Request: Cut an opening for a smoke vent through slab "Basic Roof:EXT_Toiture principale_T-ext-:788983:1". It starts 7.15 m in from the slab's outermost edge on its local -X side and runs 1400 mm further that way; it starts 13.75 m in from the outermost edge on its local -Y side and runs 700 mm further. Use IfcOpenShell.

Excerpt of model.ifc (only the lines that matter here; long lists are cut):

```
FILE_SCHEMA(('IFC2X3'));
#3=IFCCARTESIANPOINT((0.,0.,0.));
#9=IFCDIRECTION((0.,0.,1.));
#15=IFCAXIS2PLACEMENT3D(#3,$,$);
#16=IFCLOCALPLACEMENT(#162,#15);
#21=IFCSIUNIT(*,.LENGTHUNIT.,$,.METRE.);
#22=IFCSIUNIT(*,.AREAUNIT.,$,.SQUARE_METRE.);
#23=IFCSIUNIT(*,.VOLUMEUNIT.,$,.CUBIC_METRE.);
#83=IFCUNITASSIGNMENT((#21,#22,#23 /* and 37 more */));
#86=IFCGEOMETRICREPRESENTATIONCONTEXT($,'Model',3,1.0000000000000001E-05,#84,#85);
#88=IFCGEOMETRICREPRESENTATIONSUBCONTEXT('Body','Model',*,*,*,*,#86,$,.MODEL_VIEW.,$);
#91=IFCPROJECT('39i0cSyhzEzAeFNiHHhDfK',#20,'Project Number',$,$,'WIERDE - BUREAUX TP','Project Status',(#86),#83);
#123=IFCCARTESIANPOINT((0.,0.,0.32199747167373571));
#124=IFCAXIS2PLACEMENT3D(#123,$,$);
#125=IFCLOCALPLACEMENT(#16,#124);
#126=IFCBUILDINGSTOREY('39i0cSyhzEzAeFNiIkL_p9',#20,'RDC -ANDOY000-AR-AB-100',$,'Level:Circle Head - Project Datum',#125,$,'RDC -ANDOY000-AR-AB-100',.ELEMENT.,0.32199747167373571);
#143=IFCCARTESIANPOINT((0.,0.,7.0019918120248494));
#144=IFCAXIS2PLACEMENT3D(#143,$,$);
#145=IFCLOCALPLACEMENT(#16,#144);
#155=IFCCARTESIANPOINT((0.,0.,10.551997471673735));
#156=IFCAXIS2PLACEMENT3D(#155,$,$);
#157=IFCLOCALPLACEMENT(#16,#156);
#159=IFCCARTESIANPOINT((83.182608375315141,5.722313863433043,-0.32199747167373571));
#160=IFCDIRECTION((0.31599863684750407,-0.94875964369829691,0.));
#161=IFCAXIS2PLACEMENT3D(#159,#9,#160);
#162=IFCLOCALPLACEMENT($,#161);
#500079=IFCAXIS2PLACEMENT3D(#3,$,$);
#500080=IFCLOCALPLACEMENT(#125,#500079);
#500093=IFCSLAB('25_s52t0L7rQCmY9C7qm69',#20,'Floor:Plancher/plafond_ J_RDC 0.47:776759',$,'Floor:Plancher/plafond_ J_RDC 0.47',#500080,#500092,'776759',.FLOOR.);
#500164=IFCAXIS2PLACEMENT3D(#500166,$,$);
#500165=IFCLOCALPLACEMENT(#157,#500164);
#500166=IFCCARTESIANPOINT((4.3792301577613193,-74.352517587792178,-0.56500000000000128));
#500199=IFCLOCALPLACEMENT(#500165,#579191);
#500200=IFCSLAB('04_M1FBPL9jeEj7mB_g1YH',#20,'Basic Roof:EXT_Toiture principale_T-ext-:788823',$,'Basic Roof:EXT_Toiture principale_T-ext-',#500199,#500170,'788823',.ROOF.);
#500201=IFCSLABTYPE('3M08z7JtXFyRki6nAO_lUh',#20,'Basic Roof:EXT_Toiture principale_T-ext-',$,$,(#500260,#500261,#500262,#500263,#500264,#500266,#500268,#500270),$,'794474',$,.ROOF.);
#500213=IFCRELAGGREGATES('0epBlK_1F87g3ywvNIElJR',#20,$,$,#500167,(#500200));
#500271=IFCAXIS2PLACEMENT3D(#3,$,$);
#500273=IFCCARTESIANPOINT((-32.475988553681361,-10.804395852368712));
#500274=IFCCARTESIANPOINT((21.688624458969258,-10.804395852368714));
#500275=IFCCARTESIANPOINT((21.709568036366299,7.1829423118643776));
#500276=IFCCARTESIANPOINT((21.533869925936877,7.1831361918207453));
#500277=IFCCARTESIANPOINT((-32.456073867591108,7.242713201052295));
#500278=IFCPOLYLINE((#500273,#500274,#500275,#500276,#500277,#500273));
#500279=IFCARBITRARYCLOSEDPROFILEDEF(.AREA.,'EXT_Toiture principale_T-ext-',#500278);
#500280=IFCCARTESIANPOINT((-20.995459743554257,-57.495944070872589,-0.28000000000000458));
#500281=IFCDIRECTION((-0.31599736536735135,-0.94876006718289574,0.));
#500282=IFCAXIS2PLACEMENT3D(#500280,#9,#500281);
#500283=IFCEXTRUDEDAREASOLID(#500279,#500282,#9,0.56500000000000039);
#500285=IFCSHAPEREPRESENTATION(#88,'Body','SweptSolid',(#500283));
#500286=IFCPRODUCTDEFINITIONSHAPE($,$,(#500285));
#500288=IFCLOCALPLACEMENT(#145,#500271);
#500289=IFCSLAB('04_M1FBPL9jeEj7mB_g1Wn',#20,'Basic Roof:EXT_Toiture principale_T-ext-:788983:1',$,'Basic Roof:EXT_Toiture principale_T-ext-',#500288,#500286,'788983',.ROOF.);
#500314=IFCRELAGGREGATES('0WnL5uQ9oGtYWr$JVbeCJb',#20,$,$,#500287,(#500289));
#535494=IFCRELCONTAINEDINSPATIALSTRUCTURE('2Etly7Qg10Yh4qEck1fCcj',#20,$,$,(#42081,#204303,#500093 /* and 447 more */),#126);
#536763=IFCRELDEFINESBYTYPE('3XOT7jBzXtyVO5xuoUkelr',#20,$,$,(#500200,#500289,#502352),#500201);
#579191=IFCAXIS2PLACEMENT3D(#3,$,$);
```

```python
import numpy as np
import ifcopenshell
import ifcopenshell.api.feature
import ifcopenshell.api.geometry
import ifcopenshell.api.root
import ifcopenshell.geom
import ifcopenshell.util.placement
import ifcopenshell.util.representation
import ifcopenshell.util.shape
import ifcopenshell.util.unit

model = ifcopenshell.open("model.ifc")
unit_scale = ifcopenshell.util.unit.calculate_unit_scale(model)
settings = ifcopenshell.geom.settings()


def volume(element):
    """Net volume in cubic metres, openings subtracted."""
    shape = ifcopenshell.geom.create_shape(settings, element)
    return ifcopenshell.util.shape.get_volume(shape.geometry)


slab = model.by_guid("04_M1FBPL9jeEj7mB_g1Wn")
before = volume(slab)

# Extent in the slab's own axes, in metres. The edges named are its -X and -Y sides.
slab_shape = ifcopenshell.geom.create_shape(settings, slab)
vertices = ifcopenshell.util.shape.get_vertices(slab_shape.geometry)
x_min, y_min, bottom = vertices.min(axis=0)
top = vertices[:, 2].max()

opening = ifcopenshell.api.root.create_entity(model, ifc_class="IfcOpeningElement", name="Smoke vent opening")
context = ifcopenshell.util.representation.get_context(model, "Model", "Body", "MODEL_VIEW")
width, depth = 1.4, 0.7
outline = [(0.0, 0.0), (width, 0.0), (width, depth), (0.0, depth), (0.0, 0.0)]
# Overshoot both faces by 50 mm so the cut is clean.
shape = ifcopenshell.api.geometry.add_slab_representation(
    model, context=context, depth=top - bottom + 0.1, polyline=outline
)
ifcopenshell.api.geometry.assign_representation(model, product=opening, representation=shape)

matrix = ifcopenshell.util.placement.get_local_placement(slab.ObjectPlacement)
matrix[:, 3] = matrix @ np.append(np.array([x_min + 7.15, y_min + 13.75, bottom - 0.05]) / unit_scale, 1.0)
ifcopenshell.api.geometry.edit_object_placement(model, product=opening, matrix=matrix, is_si=False)
ifcopenshell.api.feature.add_feature(model, feature=opening, element=slab)

after = volume(slab)

print(f"slab volume {before:.3f} -> {after:.3f} m3")

model.write("model-out.ifc")
```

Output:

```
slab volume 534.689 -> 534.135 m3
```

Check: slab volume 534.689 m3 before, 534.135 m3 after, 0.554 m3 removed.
